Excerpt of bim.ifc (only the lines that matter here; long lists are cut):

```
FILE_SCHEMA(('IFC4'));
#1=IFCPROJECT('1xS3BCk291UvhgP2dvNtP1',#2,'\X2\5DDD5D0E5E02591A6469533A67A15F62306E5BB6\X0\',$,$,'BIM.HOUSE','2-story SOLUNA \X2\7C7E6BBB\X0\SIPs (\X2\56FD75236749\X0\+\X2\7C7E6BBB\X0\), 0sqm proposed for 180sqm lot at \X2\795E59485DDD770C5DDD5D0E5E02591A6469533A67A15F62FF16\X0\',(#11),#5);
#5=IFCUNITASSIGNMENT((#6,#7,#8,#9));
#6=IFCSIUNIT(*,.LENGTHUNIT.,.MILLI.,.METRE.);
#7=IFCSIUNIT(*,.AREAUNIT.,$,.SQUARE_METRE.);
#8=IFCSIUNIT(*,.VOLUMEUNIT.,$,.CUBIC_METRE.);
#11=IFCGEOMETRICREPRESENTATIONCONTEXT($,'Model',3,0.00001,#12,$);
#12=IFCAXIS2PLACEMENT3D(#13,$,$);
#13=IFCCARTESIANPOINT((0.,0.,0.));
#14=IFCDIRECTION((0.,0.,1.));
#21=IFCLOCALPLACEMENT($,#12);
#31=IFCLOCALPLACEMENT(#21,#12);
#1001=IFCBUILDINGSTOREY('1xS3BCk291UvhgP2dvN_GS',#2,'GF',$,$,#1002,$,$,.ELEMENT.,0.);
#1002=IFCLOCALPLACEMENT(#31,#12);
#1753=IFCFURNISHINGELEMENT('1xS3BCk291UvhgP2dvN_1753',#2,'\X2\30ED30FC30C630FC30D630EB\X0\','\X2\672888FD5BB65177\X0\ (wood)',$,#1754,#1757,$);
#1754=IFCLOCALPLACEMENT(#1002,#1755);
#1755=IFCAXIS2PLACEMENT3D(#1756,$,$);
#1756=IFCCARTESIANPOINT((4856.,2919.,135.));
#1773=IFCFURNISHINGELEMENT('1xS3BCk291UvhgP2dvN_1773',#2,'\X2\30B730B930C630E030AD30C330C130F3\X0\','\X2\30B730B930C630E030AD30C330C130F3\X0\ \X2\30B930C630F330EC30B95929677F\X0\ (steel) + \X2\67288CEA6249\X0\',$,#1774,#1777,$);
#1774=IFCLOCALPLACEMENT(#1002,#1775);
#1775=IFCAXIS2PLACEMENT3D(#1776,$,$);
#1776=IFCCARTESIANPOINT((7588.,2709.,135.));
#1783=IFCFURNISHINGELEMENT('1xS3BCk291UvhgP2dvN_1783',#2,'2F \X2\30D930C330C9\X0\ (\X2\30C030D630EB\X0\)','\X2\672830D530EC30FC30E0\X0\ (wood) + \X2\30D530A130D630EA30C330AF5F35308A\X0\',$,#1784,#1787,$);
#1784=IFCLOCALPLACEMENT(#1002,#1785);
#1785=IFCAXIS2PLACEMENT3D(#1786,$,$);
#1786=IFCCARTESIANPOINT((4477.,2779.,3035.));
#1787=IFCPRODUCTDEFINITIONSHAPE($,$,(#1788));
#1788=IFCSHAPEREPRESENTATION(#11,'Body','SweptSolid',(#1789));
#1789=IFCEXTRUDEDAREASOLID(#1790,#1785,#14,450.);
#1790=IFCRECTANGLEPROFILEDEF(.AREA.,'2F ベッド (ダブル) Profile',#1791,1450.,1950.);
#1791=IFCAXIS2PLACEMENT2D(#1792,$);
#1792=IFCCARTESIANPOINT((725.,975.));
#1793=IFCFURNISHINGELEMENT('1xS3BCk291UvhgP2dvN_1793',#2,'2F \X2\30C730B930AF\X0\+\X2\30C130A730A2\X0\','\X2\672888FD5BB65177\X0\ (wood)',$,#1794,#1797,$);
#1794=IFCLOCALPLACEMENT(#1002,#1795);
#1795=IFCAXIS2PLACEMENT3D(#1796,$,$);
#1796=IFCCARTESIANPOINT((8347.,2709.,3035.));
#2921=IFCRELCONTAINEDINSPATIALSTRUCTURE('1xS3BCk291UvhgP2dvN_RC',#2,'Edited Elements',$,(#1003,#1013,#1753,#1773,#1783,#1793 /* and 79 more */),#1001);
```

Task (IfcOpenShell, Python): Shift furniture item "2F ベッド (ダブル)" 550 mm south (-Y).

```python
import ifcopenshell
import ifcopenshell.api.geometry
import ifcopenshell.util.placement
import ifcopenshell.util.unit

model = ifcopenshell.open("bim.ifc")
unit_scale = ifcopenshell.util.unit.calculate_unit_scale(model)

item = model.by_guid("1xS3BCk291UvhgP2dvN_1783")
matrix = ifcopenshell.util.placement.get_local_placement(item.ObjectPlacement)
matrix[1, 3] -= 0.55 / unit_scale
ifcopenshell.api.geometry.edit_object_placement(model, product=item, matrix=matrix, is_si=False)

print(ifcopenshell.util.placement.get_local_placement(item.ObjectPlacement).round(3) + 0.0)

model.write("bim_updated.ifc")
```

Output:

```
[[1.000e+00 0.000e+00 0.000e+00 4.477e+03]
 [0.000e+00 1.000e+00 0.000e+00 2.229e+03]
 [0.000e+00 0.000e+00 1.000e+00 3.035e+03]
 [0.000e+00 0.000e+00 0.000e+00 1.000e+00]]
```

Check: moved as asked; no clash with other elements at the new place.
